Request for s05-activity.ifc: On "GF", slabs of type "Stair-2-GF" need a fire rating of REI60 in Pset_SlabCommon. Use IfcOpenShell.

First a look at what the model holds.

```python
import ifcopenshell
import ifcopenshell.util.element

model = ifcopenshell.open("s05-activity.ifc")
print(model.schema)
storey = next(s for s in model.by_type("IfcBuildingStorey") if s.Name == "GF")
slabs = [e for e in ifcopenshell.util.element.get_decomposition(storey) if e.is_a("IfcSlab")]
seen = {}
for e in slabs:
    element_type = ifcopenshell.util.element.get_type(e)
    key = (element_type.Name if element_type != e and element_type else None, ifcopenshell.util.element.get_pset(e, "Pset_SlabCommon", "FireRating"))
    seen[key] = seen.get(key, 0) + 1
for (name, value), count in sorted(seen.items(), key=str):
    print(count, "x", name, "|", value)
```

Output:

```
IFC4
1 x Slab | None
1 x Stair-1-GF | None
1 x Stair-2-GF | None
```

```python
import ifcopenshell
import ifcopenshell.api.pset
import ifcopenshell.util.element

model = ifcopenshell.open("s05-activity.ifc")

storey = next(s for s in model.by_type("IfcBuildingStorey") if s.Name == "GF")
slabs = [e for e in ifcopenshell.util.element.get_decomposition(storey) if e.is_a("IfcSlab")]

count = 0
for e in slabs:
    element_type = ifcopenshell.util.element.get_type(e)
    if element_type in (None, e) or element_type.Name != "Stair-2-GF":
        continue
    # add_pset returns the element's existing set when there is one.
    pset = ifcopenshell.api.pset.add_pset(model, product=e, name="Pset_SlabCommon")
    ifcopenshell.api.pset.edit_pset(model, pset=pset, properties={"FireRating": "REI60"})
    count += 1

print(count, "slabs updated")

model.write("s05-activity-out.ifc")
```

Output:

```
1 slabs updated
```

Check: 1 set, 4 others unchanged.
